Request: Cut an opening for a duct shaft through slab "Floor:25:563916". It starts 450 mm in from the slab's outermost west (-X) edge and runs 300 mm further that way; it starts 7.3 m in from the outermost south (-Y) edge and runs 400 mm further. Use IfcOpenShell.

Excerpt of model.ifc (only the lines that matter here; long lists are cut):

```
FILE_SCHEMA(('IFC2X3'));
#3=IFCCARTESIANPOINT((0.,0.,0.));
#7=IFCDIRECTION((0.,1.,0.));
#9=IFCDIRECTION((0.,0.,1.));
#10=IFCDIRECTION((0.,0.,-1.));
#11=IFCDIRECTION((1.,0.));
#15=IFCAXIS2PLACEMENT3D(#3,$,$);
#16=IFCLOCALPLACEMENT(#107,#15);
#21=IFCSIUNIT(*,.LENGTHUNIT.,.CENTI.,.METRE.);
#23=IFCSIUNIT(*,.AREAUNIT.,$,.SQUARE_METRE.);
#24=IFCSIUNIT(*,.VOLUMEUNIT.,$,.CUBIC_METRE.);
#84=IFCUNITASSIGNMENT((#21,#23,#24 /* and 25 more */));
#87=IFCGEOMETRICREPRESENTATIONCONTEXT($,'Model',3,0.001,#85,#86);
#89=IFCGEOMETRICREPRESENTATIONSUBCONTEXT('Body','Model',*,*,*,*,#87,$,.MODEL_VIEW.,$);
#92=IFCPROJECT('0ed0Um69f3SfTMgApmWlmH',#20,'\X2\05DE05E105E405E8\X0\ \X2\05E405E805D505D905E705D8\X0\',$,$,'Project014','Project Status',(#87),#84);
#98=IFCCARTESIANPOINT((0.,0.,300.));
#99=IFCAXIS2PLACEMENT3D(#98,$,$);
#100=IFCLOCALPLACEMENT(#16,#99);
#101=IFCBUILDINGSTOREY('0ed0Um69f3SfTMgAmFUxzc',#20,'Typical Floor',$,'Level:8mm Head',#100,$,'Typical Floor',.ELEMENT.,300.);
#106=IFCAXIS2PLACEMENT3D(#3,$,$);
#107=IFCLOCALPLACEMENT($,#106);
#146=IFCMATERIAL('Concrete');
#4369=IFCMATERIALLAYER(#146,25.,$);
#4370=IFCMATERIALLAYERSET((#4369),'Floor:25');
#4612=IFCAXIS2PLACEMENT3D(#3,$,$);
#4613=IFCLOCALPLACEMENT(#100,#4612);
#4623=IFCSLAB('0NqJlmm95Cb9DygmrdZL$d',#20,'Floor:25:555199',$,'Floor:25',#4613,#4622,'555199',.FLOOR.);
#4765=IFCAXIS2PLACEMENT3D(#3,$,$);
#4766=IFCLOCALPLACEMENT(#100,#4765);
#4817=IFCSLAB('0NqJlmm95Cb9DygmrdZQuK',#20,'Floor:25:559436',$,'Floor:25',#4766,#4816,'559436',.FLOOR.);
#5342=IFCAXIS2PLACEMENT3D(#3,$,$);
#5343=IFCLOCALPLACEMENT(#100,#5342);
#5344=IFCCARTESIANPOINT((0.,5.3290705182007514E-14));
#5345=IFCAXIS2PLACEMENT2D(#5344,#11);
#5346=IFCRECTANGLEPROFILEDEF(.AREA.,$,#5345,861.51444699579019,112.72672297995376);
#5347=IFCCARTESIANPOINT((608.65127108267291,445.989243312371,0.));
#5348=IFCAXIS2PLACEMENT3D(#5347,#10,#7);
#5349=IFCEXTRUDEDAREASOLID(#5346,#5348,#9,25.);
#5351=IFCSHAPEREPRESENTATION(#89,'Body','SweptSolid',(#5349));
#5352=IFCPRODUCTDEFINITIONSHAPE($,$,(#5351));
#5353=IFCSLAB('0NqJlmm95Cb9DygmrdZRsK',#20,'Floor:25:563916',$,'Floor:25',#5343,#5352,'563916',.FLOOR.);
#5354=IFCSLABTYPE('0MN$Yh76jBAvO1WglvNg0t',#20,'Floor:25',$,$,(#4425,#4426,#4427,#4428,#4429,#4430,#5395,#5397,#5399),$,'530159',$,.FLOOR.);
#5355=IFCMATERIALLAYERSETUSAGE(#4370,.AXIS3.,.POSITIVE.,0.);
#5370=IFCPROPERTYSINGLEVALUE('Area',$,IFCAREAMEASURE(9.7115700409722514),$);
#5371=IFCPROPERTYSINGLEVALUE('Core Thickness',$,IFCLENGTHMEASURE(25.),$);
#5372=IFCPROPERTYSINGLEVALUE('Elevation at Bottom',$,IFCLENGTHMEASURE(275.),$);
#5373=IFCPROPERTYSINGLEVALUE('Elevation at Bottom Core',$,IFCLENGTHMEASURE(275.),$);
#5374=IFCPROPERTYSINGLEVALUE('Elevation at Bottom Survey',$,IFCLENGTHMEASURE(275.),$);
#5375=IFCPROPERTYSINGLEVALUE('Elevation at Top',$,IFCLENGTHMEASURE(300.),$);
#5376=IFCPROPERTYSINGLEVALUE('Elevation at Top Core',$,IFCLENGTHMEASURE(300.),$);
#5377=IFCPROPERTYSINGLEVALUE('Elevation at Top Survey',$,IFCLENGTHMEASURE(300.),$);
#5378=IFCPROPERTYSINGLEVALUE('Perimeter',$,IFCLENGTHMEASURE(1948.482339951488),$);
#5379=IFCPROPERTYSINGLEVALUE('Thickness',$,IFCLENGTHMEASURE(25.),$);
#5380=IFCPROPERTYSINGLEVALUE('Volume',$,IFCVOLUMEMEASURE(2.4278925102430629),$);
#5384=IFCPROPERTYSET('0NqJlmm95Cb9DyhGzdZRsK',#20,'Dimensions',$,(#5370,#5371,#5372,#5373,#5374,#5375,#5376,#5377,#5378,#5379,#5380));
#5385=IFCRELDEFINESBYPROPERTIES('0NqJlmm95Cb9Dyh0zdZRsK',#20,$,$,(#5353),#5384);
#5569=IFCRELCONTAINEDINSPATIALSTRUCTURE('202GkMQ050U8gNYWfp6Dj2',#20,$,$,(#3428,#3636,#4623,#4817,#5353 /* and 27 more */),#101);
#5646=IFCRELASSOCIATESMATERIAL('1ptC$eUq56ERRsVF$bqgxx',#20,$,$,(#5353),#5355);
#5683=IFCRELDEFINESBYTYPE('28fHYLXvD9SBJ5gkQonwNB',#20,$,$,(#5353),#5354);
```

```python
import numpy as np
import ifcopenshell
import ifcopenshell.api.feature
import ifcopenshell.api.geometry
import ifcopenshell.api.pset
import ifcopenshell.api.root
import ifcopenshell.geom
import ifcopenshell.util.element
import ifcopenshell.util.placement
import ifcopenshell.util.representation
import ifcopenshell.util.shape
import ifcopenshell.util.unit

model = ifcopenshell.open("model.ifc")
unit_scale = ifcopenshell.util.unit.calculate_unit_scale(model)
area_scale = ifcopenshell.util.unit.calculate_unit_scale(model, "AREAUNIT")
volume_scale = ifcopenshell.util.unit.calculate_unit_scale(model, "VOLUMEUNIT")
settings = ifcopenshell.geom.settings()


def volume(element):
    """Net volume in cubic metres, openings subtracted."""
    shape = ifcopenshell.geom.create_shape(settings, element)
    return ifcopenshell.util.shape.get_volume(shape.geometry)


slab = model.by_guid("0NqJlmm95Cb9DygmrdZRsK")
before = volume(slab)

# Extent in the slab's own axes, in metres. The edges named are its -X and -Y sides.
slab_shape = ifcopenshell.geom.create_shape(settings, slab)
vertices = ifcopenshell.util.shape.get_vertices(slab_shape.geometry)
x_min, y_min, bottom = vertices.min(axis=0)
top = vertices[:, 2].max()

opening = ifcopenshell.api.root.create_entity(model, ifc_class="IfcOpeningElement", name="Duct shaft opening")
context = ifcopenshell.util.representation.get_context(model, "Model", "Body", "MODEL_VIEW")
width, depth = 0.3, 0.4
outline = [(0.0, 0.0), (width, 0.0), (width, depth), (0.0, depth), (0.0, 0.0)]
# Overshoot both faces by 50 mm so the cut is clean.
shape = ifcopenshell.api.geometry.add_slab_representation(
    model, context=context, depth=top - bottom + 0.1, polyline=outline
)
ifcopenshell.api.geometry.assign_representation(model, product=opening, representation=shape)

matrix = ifcopenshell.util.placement.get_local_placement(slab.ObjectPlacement)
matrix[:, 3] = matrix @ np.append(np.array([x_min + 0.45, y_min + 7.3, bottom - 0.05]) / unit_scale, 1.0)
ifcopenshell.api.geometry.edit_object_placement(model, product=opening, matrix=matrix, is_si=False)
ifcopenshell.api.feature.add_feature(model, feature=opening, element=slab)

after = volume(slab)

# Update the slab's stored quantities.
pset = model.by_id(ifcopenshell.util.element.get_pset(slab, "Dimensions", should_inherit=False)["id"])
ifcopenshell.api.pset.edit_pset(model, pset=pset, properties={
    "Area": model.create_entity("IfcAreaMeasure", after / (top - bottom) / area_scale),
    "Volume": model.create_entity("IfcVolumeMeasure", after / volume_scale),
})

print(f"slab volume {before:.3f} -> {after:.3f} m3")

model.write("model_rev.ifc")
```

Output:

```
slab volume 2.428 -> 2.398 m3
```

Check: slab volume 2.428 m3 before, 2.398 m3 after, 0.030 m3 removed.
